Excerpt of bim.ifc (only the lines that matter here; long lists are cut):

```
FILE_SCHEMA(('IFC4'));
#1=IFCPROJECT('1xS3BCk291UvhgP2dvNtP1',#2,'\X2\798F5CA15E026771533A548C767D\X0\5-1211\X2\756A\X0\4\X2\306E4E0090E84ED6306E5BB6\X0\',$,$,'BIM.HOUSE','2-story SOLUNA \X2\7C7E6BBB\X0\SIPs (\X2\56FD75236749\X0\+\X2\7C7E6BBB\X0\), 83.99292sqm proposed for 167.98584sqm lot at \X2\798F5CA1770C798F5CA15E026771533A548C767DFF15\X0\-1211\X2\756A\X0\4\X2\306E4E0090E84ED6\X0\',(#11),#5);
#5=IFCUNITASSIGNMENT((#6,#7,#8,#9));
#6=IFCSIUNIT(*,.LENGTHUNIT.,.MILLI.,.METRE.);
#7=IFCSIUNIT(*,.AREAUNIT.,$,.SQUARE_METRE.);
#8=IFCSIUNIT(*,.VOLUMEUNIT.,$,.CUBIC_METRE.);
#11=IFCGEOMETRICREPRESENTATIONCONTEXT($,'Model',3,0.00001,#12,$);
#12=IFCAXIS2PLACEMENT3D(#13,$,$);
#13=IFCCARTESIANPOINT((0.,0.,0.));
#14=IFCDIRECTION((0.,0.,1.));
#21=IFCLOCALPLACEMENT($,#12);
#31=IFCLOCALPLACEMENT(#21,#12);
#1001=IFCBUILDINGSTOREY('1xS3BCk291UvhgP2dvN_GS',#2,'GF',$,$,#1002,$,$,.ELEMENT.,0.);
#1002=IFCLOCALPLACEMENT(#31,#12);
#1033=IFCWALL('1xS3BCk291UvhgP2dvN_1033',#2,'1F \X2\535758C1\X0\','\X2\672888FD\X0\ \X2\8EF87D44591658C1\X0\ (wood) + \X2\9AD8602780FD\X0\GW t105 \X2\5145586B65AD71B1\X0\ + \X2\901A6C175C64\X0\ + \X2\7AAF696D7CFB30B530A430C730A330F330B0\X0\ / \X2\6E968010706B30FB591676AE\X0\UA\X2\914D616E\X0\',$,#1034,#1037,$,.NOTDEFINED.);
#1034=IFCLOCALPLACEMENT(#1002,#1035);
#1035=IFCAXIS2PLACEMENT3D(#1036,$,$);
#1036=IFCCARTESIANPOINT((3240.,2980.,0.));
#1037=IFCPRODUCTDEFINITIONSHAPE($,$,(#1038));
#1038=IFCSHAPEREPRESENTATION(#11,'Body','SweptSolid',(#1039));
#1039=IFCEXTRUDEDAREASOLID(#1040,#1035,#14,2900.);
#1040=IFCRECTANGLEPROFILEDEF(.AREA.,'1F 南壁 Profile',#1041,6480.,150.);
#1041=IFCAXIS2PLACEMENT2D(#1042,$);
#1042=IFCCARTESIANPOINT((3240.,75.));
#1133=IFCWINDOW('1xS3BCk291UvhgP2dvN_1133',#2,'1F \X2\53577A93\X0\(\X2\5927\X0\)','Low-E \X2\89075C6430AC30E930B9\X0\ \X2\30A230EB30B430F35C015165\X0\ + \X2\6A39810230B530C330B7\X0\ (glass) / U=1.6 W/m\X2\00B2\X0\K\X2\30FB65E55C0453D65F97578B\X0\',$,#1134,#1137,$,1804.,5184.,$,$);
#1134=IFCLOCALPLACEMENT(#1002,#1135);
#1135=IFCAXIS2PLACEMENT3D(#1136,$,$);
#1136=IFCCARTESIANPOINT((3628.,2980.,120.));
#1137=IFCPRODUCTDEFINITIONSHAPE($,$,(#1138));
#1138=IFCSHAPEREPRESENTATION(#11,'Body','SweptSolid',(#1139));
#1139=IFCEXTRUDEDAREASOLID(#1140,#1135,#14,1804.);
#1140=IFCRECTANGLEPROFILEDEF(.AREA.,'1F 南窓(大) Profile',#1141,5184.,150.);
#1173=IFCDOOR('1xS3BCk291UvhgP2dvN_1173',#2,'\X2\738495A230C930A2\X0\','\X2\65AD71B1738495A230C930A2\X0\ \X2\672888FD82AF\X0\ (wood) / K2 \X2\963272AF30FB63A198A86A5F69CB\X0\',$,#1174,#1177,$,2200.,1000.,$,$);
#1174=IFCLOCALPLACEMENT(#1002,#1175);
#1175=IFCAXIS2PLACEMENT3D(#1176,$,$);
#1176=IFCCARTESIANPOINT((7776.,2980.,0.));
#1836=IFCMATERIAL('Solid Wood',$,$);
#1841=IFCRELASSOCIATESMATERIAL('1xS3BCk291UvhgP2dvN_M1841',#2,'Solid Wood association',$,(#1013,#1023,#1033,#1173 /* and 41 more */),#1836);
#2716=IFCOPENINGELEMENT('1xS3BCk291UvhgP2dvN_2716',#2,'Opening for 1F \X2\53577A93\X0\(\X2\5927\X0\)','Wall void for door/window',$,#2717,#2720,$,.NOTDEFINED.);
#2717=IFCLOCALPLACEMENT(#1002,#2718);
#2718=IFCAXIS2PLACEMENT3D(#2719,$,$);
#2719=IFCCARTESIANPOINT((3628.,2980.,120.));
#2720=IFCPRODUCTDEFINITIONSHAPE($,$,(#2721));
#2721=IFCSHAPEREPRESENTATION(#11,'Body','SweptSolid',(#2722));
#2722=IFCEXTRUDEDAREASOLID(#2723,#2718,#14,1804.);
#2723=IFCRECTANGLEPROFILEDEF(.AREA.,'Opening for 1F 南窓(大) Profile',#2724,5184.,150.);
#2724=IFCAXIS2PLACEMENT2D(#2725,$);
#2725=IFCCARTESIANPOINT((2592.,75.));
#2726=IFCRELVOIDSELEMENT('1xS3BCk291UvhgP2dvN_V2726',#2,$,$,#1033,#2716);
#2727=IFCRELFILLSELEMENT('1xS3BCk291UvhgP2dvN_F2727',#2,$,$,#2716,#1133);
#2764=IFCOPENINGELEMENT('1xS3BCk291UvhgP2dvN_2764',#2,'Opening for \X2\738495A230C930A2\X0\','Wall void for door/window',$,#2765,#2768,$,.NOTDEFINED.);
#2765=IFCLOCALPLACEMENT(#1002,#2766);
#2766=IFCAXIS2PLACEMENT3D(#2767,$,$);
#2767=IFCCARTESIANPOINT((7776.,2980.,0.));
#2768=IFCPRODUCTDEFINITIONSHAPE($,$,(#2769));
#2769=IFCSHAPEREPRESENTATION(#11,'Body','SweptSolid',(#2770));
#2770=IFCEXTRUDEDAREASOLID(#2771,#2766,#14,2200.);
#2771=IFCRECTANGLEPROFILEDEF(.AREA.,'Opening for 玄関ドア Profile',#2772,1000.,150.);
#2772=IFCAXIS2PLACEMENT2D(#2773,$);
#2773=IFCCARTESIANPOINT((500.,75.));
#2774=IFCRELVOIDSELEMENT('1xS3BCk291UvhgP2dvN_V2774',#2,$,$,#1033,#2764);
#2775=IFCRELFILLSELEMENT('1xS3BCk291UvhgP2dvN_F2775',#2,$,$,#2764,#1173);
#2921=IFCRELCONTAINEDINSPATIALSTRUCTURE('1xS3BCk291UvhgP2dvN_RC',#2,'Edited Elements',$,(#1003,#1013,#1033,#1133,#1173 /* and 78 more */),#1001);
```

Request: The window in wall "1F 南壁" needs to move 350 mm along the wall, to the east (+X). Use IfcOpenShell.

```python
import ifcopenshell
import ifcopenshell.api.geometry
import ifcopenshell.util.placement
import ifcopenshell.util.unit

model = ifcopenshell.open("bim.ifc")
unit_scale = ifcopenshell.util.unit.calculate_unit_scale(model)

window = model.by_guid("1xS3BCk291UvhgP2dvN_1133")
opening = window.FillsVoids[0].RelatingOpeningElement
wall = opening.VoidsElements[0].RelatingBuildingElement

wall_matrix = ifcopenshell.util.placement.get_local_placement(wall.ObjectPlacement)
shift = wall_matrix[:3, 0] * 0.35 / unit_scale
before = ifcopenshell.util.placement.get_local_placement(window.ObjectPlacement)[:3, 3].copy()

# The window is not placed relative to its opening, so move both.
for product in (opening, window):
    matrix = ifcopenshell.util.placement.get_local_placement(product.ObjectPlacement)
    matrix[:3, 3] += shift
    ifcopenshell.api.geometry.edit_object_placement(model, product=product, matrix=matrix, is_si=False)

after = ifcopenshell.util.placement.get_local_placement(window.ObjectPlacement)[:3, 3]
print("window moved by", (after - before).round(3) + 0.0)

model.write("bim_edited.ifc")
```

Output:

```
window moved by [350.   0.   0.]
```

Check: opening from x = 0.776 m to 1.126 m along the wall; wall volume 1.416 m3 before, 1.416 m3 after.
